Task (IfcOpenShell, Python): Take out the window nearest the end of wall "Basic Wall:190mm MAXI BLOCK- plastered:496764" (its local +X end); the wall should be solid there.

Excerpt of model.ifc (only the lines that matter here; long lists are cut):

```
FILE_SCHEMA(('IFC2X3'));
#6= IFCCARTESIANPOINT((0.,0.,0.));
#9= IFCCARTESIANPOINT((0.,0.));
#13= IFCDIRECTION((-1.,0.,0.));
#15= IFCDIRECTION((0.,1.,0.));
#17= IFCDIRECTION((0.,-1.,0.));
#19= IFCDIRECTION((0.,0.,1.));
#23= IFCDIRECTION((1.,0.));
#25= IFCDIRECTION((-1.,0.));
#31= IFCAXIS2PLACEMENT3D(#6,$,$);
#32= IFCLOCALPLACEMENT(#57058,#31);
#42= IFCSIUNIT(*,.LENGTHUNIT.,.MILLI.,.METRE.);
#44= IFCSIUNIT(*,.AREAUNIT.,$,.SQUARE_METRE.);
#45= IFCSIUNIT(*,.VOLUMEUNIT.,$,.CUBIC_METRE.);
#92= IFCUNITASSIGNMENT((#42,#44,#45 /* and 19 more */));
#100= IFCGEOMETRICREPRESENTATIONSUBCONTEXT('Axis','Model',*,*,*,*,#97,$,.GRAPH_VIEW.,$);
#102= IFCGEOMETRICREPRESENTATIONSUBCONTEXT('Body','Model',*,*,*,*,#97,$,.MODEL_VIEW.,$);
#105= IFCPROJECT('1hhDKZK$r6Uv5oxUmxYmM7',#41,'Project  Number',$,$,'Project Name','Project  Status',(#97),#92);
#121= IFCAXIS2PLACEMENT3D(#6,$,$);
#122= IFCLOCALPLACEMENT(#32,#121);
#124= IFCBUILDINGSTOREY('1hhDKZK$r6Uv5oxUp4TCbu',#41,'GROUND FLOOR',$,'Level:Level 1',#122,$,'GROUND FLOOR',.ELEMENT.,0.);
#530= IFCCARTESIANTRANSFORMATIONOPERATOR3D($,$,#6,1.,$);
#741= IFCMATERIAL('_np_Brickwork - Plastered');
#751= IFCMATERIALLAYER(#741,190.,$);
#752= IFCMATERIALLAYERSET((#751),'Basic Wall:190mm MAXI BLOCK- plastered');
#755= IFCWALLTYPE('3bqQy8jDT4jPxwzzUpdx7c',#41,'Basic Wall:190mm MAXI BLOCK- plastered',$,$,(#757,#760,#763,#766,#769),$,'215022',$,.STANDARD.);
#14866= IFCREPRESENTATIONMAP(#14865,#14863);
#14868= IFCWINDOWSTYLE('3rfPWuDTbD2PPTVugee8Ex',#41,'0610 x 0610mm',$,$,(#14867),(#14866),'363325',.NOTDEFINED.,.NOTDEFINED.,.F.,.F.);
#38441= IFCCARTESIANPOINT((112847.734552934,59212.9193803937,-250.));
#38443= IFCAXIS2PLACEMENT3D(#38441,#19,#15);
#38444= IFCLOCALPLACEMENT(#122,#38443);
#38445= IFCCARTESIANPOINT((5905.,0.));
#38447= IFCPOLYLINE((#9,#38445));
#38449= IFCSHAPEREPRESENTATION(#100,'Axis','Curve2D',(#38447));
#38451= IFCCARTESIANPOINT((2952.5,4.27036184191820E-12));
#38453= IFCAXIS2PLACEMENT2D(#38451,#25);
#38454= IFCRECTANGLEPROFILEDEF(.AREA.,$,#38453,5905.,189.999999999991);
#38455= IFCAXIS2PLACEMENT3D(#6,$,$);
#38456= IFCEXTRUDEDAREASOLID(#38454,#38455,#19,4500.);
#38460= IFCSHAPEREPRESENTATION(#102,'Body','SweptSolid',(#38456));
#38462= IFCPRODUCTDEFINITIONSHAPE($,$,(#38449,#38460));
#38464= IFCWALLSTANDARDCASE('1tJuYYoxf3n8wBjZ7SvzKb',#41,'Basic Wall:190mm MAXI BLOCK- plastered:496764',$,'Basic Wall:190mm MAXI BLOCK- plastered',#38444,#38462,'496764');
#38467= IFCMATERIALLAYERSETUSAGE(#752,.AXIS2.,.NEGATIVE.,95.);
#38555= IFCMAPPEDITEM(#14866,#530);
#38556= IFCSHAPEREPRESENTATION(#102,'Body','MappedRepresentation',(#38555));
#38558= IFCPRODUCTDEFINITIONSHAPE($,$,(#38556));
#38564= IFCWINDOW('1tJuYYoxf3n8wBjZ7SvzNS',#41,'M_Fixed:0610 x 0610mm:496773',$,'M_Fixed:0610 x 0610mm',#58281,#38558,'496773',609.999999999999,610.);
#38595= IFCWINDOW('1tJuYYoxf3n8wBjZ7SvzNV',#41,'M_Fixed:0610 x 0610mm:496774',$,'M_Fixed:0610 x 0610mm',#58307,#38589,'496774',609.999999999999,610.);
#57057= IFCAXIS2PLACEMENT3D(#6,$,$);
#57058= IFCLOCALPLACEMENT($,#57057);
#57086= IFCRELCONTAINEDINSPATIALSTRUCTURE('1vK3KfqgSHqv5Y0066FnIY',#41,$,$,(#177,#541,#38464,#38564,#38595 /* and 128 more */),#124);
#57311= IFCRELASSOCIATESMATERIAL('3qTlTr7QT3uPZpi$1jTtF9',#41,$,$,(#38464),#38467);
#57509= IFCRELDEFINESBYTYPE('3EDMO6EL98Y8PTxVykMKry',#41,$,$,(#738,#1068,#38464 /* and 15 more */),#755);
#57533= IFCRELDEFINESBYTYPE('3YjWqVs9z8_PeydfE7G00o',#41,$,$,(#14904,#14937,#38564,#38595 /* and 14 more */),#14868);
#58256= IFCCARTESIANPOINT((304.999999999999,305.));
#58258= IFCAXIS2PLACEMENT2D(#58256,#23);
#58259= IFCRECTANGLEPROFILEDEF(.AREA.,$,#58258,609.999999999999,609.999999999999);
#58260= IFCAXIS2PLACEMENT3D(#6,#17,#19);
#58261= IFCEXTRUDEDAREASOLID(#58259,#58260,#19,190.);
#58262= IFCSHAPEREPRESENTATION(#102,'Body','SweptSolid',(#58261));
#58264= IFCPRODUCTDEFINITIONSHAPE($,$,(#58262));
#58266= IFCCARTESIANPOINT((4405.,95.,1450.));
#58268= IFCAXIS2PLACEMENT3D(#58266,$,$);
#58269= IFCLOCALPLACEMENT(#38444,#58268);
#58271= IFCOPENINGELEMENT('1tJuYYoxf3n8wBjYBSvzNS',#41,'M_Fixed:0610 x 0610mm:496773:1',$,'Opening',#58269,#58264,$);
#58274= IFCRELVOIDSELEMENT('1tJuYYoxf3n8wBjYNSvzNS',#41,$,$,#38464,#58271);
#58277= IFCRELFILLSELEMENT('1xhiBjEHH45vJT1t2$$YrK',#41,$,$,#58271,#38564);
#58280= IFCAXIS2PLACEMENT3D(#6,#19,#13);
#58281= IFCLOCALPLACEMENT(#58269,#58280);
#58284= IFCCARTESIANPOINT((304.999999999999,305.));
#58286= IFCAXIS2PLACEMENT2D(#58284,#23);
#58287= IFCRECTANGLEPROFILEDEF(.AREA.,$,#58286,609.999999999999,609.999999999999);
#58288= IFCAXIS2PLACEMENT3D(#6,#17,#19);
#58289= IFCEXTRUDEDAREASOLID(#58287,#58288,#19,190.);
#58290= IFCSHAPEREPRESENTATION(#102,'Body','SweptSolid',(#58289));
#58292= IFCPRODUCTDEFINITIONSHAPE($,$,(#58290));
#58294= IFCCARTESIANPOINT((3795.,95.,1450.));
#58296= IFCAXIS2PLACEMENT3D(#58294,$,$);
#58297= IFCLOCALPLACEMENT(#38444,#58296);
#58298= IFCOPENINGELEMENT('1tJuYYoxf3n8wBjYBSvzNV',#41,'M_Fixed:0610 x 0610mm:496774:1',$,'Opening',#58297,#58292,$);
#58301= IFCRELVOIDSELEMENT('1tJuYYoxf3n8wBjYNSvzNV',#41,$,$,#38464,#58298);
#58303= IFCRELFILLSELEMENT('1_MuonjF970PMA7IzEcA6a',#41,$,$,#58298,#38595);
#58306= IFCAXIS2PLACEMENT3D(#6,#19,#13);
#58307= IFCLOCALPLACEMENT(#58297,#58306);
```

```python
import ifcopenshell
import ifcopenshell.api.feature
import ifcopenshell.api.root
import ifcopenshell.geom
import ifcopenshell.util.shape

model = ifcopenshell.open("model.ifc")
settings = ifcopenshell.geom.settings()


def volume(element):
    """Net volume in cubic metres, openings subtracted."""
    shape = ifcopenshell.geom.create_shape(settings, element)
    return ifcopenshell.util.shape.get_volume(shape.geometry)


window = model.by_guid("1tJuYYoxf3n8wBjZ7SvzNS")
opening = window.FillsVoids[0].RelatingOpeningElement
wall = opening.VoidsElements[0].RelatingBuildingElement
before = volume(wall)

ifcopenshell.api.root.remove_product(model, product=window)
ifcopenshell.api.feature.remove_feature(model, feature=opening)

after = volume(wall)

print(f"wall volume {before:.3f} -> {after:.3f} m3")

model.write("model_v2.ifc")
```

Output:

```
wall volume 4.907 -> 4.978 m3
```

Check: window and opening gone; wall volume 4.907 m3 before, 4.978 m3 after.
